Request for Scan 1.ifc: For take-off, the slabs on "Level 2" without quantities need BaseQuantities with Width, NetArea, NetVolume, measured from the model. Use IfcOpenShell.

First a look at what the model holds.

```python
import ifcopenshell
import ifcopenshell.util.element
import ifcopenshell.util.unit

model = ifcopenshell.open("Scan 1.ifc")
print(model.schema)
for unit_type in ("LENGTHUNIT", "AREAUNIT", "VOLUMEUNIT"):
    print(unit_type, ifcopenshell.util.unit.calculate_unit_scale(model, unit_type))
storey = next(s for s in model.by_type("IfcBuildingStorey") if s.Name == "Level 2")
slabs = [e for e in ifcopenshell.util.element.get_decomposition(storey) if e.is_a("IfcSlab")]
for e in sorted(slabs, key=lambda e: e.id()):
    print(e.id(), e.is_a(), e.Name, list(ifcopenshell.util.element.get_psets(e, qtos_only=True)), sep=" | ")
```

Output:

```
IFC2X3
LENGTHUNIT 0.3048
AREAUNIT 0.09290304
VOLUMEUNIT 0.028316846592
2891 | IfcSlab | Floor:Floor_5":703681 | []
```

```python
import ifcopenshell
import ifcopenshell.api.pset
import ifcopenshell.geom
import ifcopenshell.util.element
import ifcopenshell.util.shape
import ifcopenshell.util.unit

model = ifcopenshell.open("Scan 1.ifc")
unit_scale = ifcopenshell.util.unit.calculate_unit_scale(model)
area_scale = ifcopenshell.util.unit.calculate_unit_scale(model, "AREAUNIT")
volume_scale = ifcopenshell.util.unit.calculate_unit_scale(model, "VOLUMEUNIT")
settings = ifcopenshell.geom.settings()

storey = next(s for s in model.by_type("IfcBuildingStorey") if s.Name == "Level 2")
slabs = [e for e in ifcopenshell.util.element.get_decomposition(storey) if e.is_a("IfcSlab")]

for e in sorted(slabs, key=lambda e: e.id()):
    if ifcopenshell.util.element.get_psets(e, qtos_only=True, should_inherit=False):
        continue
    # Geometry comes back in metres, in the element's own axes.
    shape = ifcopenshell.geom.create_shape(settings, e)
    values = {
        "Width": ifcopenshell.util.shape.get_z(shape.geometry) / unit_scale,
        "NetArea": ifcopenshell.util.shape.get_footprint_area(shape.geometry) / area_scale,
        "NetVolume": ifcopenshell.util.shape.get_volume(shape.geometry) / volume_scale,
    }
    qto = ifcopenshell.api.pset.add_qto(model, product=e, name="BaseQuantities")
    ifcopenshell.api.pset.edit_qto(model, qto=qto, properties=values)
    print(e.id(), {k: round(v, 3) for k, v in values.items()})

model.write("Scan 1-out.ifc")
```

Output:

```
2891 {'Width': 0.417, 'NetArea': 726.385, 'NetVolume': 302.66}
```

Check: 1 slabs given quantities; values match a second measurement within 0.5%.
